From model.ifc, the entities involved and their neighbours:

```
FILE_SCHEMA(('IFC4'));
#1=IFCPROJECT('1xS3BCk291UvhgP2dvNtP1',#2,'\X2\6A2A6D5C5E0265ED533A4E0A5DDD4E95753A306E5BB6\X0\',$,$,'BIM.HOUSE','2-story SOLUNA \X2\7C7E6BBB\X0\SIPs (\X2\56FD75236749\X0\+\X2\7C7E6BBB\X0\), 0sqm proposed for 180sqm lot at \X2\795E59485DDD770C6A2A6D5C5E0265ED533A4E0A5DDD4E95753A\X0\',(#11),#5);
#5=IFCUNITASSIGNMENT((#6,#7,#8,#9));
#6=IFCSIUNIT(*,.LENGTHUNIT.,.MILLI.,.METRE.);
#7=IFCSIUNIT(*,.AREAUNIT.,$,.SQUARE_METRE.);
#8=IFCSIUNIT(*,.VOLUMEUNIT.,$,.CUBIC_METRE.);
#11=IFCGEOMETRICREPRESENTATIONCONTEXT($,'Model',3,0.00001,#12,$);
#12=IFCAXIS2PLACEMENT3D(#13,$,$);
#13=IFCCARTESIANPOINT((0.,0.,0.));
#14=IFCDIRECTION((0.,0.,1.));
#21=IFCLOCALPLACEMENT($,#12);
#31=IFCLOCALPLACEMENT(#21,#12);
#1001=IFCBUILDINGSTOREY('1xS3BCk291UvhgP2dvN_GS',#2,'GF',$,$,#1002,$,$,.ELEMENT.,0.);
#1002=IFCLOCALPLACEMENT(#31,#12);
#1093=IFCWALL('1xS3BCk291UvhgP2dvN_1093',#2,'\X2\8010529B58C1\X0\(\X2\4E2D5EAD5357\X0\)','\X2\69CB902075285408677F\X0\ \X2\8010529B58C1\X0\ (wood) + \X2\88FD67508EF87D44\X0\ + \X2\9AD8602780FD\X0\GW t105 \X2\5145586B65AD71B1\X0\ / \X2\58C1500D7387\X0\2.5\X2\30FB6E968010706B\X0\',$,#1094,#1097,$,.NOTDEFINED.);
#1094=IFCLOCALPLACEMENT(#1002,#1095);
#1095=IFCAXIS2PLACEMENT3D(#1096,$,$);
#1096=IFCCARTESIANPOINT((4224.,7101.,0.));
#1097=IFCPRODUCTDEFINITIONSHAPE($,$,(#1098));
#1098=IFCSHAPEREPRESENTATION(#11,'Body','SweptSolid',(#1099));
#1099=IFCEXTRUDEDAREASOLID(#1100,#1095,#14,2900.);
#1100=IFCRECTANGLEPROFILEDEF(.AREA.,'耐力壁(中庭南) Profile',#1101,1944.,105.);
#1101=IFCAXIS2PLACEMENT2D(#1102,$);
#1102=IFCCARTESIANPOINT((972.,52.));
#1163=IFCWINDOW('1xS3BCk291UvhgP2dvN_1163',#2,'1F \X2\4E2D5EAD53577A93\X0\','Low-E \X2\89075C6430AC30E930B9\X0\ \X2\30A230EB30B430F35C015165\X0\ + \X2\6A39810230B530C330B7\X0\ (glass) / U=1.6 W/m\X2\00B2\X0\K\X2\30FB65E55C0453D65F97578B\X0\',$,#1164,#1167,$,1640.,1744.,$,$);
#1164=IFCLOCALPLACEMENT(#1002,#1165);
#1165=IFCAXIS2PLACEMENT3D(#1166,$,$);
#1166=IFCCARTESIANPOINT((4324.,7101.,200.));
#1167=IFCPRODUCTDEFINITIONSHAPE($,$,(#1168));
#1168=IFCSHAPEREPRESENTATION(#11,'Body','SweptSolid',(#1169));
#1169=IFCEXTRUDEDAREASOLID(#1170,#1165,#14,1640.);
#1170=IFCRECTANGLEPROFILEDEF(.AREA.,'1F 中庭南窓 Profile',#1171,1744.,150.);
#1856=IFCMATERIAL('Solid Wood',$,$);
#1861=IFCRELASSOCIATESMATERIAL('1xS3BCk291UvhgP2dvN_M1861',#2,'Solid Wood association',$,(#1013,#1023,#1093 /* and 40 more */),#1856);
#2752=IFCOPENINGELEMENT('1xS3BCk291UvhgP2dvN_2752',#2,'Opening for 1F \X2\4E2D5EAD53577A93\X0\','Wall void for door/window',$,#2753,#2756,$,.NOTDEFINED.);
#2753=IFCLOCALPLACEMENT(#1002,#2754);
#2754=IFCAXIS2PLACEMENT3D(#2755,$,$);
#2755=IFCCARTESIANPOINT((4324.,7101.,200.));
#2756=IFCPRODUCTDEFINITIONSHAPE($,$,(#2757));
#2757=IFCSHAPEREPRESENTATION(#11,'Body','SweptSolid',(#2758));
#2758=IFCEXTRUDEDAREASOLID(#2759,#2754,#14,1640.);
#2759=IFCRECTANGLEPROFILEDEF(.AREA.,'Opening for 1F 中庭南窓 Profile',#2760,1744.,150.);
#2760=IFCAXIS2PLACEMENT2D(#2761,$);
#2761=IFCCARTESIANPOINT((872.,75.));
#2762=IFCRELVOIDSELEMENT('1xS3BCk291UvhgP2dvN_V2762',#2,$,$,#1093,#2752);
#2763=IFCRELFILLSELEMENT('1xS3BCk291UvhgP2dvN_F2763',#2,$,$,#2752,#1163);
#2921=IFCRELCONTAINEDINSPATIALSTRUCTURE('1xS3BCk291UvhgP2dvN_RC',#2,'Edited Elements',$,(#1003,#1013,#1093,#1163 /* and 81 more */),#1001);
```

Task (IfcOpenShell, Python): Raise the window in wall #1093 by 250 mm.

```python
import numpy as np
import ifcopenshell
import ifcopenshell.api.geometry
import ifcopenshell.util.placement
import ifcopenshell.util.unit

model = ifcopenshell.open("model.ifc")
unit_scale = ifcopenshell.util.unit.calculate_unit_scale(model)

window = model.by_id(1163)
opening = window.FillsVoids[0].RelatingOpeningElement
dz = 0.25 / unit_scale

shift = np.array([0.0, 0.0, dz])
# The window is not placed relative to its opening, so move both.
for product in (opening, window):
    matrix = ifcopenshell.util.placement.get_local_placement(product.ObjectPlacement)
    matrix[:3, 3] += shift
    ifcopenshell.api.geometry.edit_object_placement(model, product=product, matrix=matrix, is_si=False)

print(f"moved by {dz * unit_scale:+.3f} m")

model.write("model_edited.ifc")
```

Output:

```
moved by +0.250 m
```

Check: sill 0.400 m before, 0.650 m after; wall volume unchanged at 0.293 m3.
